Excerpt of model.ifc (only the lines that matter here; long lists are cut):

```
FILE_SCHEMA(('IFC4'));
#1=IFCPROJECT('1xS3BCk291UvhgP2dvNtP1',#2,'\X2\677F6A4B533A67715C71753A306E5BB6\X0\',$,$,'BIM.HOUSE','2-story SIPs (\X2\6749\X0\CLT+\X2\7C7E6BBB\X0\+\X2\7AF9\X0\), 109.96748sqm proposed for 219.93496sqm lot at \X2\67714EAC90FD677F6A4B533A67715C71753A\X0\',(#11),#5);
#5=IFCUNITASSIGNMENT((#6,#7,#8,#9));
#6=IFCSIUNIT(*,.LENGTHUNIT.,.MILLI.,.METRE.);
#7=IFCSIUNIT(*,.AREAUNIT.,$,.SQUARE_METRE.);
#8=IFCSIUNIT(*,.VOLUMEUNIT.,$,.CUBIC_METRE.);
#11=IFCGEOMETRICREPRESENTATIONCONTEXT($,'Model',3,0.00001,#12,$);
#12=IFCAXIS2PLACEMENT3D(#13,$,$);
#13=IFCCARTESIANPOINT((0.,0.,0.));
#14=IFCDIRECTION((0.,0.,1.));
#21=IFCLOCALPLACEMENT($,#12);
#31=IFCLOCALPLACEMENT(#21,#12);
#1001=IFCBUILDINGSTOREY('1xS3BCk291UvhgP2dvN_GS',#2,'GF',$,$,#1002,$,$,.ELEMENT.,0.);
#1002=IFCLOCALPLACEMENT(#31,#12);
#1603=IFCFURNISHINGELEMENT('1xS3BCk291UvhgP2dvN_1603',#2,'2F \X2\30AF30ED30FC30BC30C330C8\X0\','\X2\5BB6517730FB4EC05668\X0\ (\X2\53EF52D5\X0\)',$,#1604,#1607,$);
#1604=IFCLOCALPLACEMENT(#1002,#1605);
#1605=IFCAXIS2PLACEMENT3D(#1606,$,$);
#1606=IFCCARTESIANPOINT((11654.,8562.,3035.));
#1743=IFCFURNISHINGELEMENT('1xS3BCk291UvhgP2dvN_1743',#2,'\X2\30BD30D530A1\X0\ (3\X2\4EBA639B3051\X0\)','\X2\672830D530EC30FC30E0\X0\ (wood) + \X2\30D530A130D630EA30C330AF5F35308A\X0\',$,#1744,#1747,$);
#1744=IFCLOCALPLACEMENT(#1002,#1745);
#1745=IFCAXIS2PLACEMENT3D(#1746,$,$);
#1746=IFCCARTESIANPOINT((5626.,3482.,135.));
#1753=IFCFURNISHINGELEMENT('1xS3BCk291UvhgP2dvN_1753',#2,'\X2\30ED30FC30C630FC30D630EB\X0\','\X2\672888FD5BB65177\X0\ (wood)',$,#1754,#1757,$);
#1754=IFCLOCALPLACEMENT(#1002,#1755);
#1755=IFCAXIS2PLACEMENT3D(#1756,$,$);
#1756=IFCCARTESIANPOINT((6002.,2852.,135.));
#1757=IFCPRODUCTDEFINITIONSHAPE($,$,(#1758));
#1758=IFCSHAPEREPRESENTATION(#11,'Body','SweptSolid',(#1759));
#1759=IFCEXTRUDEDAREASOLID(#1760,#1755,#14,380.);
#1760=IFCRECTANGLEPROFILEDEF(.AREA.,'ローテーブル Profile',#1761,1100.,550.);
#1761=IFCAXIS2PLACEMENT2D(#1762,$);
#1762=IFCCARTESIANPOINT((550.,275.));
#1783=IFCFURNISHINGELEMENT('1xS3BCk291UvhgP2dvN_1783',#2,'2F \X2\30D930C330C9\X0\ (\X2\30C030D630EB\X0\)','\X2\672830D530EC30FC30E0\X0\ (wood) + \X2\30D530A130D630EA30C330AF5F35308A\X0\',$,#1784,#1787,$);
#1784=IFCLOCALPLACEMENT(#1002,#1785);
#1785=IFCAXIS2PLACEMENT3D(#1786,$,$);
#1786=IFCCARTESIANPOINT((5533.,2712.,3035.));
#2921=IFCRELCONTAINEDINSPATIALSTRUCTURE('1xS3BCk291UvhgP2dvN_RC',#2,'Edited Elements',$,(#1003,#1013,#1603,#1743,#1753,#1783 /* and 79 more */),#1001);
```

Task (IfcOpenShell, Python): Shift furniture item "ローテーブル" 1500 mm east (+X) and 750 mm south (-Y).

```python
import ifcopenshell
import ifcopenshell.api.geometry
import ifcopenshell.util.placement

model = ifcopenshell.open("model.ifc")

item = model.by_id(1753)
matrix = ifcopenshell.util.placement.get_local_placement(item.ObjectPlacement)
matrix[0, 3] += 1500.0
matrix[1, 3] -= 750.0
ifcopenshell.api.geometry.edit_object_placement(model, product=item, matrix=matrix, is_si=False)

print(ifcopenshell.util.placement.get_local_placement(item.ObjectPlacement).round(3) + 0.0)

model.write("model_rev.ifc")
```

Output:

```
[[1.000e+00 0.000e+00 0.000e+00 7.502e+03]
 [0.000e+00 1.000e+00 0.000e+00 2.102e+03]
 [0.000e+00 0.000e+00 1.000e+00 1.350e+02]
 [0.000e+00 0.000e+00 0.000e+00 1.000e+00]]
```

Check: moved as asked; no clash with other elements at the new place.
